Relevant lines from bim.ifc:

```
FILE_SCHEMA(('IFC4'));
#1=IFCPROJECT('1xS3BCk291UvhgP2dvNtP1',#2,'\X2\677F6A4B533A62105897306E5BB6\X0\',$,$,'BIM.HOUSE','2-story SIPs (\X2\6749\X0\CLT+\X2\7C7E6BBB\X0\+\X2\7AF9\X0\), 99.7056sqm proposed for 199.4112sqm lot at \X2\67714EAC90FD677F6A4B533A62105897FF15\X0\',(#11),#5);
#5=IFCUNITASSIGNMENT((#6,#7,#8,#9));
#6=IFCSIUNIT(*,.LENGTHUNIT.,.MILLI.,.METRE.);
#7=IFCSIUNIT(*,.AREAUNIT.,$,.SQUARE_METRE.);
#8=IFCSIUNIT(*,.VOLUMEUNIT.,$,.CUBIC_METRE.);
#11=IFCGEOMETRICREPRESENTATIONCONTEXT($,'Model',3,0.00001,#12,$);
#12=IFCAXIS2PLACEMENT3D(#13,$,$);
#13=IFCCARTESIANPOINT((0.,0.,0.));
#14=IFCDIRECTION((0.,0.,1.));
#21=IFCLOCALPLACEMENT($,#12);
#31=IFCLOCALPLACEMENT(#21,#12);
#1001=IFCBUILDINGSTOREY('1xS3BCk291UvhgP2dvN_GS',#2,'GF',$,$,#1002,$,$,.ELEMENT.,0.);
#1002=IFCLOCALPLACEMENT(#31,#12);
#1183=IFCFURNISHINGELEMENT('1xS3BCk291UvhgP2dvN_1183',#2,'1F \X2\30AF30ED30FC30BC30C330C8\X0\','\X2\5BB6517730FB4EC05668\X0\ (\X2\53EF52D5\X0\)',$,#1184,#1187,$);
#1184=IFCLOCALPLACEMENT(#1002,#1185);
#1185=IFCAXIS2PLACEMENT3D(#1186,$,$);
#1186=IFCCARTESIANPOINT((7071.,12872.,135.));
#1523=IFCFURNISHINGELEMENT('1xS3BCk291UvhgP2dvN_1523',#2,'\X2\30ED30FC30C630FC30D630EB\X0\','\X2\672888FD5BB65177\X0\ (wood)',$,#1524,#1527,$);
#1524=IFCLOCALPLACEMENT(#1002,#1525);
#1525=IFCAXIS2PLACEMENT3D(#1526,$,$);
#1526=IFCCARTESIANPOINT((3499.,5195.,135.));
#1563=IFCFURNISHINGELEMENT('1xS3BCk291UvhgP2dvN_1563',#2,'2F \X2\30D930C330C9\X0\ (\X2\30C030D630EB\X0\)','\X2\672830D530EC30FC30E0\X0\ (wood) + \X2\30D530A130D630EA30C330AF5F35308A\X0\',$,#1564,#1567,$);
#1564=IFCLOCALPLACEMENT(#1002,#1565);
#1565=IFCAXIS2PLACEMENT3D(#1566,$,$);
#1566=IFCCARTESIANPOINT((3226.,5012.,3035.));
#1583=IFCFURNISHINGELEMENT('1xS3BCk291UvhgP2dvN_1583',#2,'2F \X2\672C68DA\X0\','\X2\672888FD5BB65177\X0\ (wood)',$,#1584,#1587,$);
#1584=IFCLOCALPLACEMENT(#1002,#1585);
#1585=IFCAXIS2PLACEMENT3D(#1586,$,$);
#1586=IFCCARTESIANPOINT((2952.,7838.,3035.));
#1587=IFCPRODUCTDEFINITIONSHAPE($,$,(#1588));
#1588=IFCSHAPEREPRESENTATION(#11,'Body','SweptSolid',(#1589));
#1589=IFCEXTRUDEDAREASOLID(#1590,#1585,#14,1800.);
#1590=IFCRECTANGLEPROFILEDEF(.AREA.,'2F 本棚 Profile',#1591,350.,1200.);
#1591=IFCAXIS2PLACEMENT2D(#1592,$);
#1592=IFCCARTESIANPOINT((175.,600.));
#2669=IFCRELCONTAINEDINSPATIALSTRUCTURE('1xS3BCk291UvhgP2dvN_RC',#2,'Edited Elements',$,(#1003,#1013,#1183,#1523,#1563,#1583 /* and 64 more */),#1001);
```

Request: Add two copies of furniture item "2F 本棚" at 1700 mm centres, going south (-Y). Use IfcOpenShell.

```python
import numpy as np
import ifcopenshell
import ifcopenshell.api.geometry
import ifcopenshell.api.root
import ifcopenshell.util.element
import ifcopenshell.util.placement
import ifcopenshell.util.unit

model = ifcopenshell.open("bim.ifc")
unit_scale = ifcopenshell.util.unit.calculate_unit_scale(model)


def reuse_history(source, copy):
    """copy_class also copies each property set's owner history, people and application; keep the originals."""
    for rel in copy.IsDefinedBy:
        if rel.is_a("IfcRelDefinesByProperties") and (history := rel.RelatingPropertyDefinition.OwnerHistory):
            rel.RelatingPropertyDefinition.OwnerHistory = source.OwnerHistory
            ifcopenshell.util.element.remove_deep2(model, history)


source = model.by_guid("1xS3BCk291UvhgP2dvN_1583")
base = ifcopenshell.util.placement.get_local_placement(source.ObjectPlacement)
step = np.array([0.0, -1.0, 0.0]) * 1.7 / unit_scale

for i in range(1, 3):
    copy = ifcopenshell.api.root.copy_class(model, product=source)
    copy.Representation = ifcopenshell.util.element.copy_deep(
        model, source.Representation, exclude=["IfcGeometricRepresentationContext", "IfcRepresentationMap"]
    )
    reuse_history(source, copy)
    matrix = base.copy()
    matrix[:3, 3] += i * step
    print("added at", matrix[:3, 3].round(3) + 0.0)
    ifcopenshell.api.geometry.edit_object_placement(model, product=copy, matrix=matrix, is_si=False)

model.write("bim-out.ifc")
```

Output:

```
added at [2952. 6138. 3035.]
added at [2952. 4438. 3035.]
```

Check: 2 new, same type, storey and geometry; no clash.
